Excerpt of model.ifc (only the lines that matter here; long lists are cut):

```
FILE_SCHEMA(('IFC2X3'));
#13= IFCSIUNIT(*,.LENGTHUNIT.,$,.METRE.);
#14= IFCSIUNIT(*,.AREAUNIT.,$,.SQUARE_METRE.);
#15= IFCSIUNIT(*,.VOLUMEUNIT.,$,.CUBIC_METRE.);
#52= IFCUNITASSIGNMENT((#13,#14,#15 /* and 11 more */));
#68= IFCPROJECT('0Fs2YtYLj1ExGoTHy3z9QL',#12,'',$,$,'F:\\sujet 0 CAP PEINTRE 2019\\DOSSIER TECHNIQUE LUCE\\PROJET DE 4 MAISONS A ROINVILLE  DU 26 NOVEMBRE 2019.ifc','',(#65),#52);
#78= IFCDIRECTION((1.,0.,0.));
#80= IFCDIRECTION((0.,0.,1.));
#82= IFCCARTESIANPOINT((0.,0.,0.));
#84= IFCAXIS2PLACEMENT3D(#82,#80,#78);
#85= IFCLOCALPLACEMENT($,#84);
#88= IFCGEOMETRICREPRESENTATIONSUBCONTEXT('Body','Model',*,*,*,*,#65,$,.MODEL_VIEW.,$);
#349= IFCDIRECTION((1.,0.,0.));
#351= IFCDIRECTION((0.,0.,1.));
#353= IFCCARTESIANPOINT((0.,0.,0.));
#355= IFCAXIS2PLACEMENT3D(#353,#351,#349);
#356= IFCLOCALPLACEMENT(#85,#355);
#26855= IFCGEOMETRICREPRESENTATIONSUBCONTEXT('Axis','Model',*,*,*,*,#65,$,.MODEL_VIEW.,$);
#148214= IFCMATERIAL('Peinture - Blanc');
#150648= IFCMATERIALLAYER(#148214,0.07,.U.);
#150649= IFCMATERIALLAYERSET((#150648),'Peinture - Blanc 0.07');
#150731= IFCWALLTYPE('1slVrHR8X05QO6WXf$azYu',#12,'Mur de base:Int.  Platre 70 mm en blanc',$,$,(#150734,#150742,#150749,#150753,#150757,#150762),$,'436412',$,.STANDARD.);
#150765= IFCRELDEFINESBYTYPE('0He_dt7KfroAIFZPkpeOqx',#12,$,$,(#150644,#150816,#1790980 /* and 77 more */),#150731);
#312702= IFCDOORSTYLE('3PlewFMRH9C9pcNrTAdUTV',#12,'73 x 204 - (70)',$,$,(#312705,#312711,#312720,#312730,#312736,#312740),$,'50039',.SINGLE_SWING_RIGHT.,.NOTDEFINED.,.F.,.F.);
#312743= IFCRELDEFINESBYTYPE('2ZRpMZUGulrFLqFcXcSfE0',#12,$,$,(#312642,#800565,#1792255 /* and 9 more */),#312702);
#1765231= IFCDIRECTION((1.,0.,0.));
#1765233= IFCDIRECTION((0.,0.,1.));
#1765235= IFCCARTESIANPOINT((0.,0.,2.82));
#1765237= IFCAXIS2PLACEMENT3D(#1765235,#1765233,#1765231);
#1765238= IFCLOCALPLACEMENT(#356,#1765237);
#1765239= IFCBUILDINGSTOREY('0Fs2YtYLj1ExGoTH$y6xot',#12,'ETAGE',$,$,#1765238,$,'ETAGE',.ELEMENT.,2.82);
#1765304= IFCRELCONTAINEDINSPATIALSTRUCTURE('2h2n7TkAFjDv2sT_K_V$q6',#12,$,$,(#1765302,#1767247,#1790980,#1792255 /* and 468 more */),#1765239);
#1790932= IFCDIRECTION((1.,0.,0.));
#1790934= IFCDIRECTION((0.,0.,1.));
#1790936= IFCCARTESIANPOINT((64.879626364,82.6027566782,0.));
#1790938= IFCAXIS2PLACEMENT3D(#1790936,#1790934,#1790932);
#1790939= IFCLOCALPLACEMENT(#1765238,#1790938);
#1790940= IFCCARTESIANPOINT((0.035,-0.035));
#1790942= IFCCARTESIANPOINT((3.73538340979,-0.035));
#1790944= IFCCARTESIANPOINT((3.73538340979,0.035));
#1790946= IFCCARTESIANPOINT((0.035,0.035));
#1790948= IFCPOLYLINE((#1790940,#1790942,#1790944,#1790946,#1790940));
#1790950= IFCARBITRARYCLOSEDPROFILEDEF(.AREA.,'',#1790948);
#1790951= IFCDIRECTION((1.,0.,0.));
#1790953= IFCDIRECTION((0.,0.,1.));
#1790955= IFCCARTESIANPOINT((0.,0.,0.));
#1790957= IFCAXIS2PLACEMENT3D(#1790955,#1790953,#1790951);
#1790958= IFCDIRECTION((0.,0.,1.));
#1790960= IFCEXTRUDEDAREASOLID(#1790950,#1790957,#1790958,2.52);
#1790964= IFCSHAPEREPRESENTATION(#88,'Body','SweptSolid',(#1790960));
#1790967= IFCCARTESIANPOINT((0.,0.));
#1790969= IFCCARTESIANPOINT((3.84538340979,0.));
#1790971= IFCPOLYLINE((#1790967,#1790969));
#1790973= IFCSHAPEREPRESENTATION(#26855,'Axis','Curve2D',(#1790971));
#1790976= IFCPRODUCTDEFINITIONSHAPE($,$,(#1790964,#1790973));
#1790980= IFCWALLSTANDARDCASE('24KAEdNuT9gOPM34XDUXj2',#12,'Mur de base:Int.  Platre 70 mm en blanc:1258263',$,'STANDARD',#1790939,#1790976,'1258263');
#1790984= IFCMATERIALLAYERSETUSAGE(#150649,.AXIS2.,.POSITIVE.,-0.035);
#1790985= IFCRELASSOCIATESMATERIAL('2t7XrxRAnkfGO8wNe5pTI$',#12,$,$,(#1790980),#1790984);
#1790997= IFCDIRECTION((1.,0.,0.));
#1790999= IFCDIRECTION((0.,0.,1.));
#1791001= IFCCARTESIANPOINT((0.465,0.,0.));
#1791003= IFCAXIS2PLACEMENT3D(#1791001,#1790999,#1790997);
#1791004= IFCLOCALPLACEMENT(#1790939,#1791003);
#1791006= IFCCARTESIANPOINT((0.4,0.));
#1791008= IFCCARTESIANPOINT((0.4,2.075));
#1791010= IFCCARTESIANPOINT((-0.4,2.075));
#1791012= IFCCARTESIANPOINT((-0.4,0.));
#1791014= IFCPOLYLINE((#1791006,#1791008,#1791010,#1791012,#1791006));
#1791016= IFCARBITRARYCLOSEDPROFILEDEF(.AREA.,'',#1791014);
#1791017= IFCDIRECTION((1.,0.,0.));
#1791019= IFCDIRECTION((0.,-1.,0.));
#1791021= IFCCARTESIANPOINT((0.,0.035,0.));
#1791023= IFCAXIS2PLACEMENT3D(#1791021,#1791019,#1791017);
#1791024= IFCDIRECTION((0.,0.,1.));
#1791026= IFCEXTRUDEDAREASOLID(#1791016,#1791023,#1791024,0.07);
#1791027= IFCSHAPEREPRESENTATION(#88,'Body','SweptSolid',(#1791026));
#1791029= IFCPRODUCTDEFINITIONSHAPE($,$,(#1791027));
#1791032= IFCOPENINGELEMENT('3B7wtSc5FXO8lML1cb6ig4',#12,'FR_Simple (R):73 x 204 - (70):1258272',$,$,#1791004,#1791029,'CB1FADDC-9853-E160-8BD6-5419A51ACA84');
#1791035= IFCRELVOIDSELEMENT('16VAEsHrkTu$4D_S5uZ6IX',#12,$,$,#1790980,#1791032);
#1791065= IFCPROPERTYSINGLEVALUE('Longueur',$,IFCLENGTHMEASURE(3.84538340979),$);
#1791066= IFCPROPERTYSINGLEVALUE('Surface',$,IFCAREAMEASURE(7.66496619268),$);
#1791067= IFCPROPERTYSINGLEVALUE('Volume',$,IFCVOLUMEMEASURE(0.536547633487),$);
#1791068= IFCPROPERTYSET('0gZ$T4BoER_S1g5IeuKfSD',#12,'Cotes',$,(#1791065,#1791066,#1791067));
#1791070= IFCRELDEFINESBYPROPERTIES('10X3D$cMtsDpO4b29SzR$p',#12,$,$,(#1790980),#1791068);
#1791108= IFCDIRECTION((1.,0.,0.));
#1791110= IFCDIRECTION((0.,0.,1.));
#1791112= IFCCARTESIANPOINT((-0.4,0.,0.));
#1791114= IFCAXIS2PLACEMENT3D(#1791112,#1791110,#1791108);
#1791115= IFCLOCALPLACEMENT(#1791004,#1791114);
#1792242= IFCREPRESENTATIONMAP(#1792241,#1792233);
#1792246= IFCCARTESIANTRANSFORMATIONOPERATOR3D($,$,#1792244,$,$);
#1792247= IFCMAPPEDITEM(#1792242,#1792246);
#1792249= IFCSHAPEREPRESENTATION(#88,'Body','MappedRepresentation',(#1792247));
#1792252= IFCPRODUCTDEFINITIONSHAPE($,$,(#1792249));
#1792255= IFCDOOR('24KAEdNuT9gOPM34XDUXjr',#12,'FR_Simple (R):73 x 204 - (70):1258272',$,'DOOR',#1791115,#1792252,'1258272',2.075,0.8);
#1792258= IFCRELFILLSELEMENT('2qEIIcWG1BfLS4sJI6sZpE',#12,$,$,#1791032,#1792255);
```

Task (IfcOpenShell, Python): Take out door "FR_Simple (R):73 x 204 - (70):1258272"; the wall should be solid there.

```python
import ifcopenshell
import ifcopenshell.api.feature
import ifcopenshell.api.pset
import ifcopenshell.api.root
import ifcopenshell.geom
import ifcopenshell.util.element
import ifcopenshell.util.shape
import ifcopenshell.util.unit

model = ifcopenshell.open("model.ifc")
area_scale = ifcopenshell.util.unit.calculate_unit_scale(model, "AREAUNIT")
volume_scale = ifcopenshell.util.unit.calculate_unit_scale(model, "VOLUMEUNIT")
settings = ifcopenshell.geom.settings()


def volume(element):
    """Net volume in cubic metres, openings subtracted."""
    shape = ifcopenshell.geom.create_shape(settings, element)
    return ifcopenshell.util.shape.get_volume(shape.geometry)


door = model.by_guid("24KAEdNuT9gOPM34XDUXjr")
opening = door.FillsVoids[0].RelatingOpeningElement
wall = opening.VoidsElements[0].RelatingBuildingElement
before = volume(wall)

ifcopenshell.api.root.remove_product(model, product=door)
ifcopenshell.api.feature.remove_feature(model, feature=opening)

after = volume(wall)
thickness = 0.07  # wall thickness in metres

# Update the wall's stored quantities.
pset = model.by_id(ifcopenshell.util.element.get_pset(wall, "Cotes", should_inherit=False)["id"])
ifcopenshell.api.pset.edit_pset(model, pset=pset, properties={
    "Surface": model.create_entity("IfcAreaMeasure", after / thickness / area_scale),
    "Volume": model.create_entity("IfcVolumeMeasure", after / volume_scale),
})

print(f"wall volume {before:.3f} -> {after:.3f} m3")

model.write("model_rev.ifc")
```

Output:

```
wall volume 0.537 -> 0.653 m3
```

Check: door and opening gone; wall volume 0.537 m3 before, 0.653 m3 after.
